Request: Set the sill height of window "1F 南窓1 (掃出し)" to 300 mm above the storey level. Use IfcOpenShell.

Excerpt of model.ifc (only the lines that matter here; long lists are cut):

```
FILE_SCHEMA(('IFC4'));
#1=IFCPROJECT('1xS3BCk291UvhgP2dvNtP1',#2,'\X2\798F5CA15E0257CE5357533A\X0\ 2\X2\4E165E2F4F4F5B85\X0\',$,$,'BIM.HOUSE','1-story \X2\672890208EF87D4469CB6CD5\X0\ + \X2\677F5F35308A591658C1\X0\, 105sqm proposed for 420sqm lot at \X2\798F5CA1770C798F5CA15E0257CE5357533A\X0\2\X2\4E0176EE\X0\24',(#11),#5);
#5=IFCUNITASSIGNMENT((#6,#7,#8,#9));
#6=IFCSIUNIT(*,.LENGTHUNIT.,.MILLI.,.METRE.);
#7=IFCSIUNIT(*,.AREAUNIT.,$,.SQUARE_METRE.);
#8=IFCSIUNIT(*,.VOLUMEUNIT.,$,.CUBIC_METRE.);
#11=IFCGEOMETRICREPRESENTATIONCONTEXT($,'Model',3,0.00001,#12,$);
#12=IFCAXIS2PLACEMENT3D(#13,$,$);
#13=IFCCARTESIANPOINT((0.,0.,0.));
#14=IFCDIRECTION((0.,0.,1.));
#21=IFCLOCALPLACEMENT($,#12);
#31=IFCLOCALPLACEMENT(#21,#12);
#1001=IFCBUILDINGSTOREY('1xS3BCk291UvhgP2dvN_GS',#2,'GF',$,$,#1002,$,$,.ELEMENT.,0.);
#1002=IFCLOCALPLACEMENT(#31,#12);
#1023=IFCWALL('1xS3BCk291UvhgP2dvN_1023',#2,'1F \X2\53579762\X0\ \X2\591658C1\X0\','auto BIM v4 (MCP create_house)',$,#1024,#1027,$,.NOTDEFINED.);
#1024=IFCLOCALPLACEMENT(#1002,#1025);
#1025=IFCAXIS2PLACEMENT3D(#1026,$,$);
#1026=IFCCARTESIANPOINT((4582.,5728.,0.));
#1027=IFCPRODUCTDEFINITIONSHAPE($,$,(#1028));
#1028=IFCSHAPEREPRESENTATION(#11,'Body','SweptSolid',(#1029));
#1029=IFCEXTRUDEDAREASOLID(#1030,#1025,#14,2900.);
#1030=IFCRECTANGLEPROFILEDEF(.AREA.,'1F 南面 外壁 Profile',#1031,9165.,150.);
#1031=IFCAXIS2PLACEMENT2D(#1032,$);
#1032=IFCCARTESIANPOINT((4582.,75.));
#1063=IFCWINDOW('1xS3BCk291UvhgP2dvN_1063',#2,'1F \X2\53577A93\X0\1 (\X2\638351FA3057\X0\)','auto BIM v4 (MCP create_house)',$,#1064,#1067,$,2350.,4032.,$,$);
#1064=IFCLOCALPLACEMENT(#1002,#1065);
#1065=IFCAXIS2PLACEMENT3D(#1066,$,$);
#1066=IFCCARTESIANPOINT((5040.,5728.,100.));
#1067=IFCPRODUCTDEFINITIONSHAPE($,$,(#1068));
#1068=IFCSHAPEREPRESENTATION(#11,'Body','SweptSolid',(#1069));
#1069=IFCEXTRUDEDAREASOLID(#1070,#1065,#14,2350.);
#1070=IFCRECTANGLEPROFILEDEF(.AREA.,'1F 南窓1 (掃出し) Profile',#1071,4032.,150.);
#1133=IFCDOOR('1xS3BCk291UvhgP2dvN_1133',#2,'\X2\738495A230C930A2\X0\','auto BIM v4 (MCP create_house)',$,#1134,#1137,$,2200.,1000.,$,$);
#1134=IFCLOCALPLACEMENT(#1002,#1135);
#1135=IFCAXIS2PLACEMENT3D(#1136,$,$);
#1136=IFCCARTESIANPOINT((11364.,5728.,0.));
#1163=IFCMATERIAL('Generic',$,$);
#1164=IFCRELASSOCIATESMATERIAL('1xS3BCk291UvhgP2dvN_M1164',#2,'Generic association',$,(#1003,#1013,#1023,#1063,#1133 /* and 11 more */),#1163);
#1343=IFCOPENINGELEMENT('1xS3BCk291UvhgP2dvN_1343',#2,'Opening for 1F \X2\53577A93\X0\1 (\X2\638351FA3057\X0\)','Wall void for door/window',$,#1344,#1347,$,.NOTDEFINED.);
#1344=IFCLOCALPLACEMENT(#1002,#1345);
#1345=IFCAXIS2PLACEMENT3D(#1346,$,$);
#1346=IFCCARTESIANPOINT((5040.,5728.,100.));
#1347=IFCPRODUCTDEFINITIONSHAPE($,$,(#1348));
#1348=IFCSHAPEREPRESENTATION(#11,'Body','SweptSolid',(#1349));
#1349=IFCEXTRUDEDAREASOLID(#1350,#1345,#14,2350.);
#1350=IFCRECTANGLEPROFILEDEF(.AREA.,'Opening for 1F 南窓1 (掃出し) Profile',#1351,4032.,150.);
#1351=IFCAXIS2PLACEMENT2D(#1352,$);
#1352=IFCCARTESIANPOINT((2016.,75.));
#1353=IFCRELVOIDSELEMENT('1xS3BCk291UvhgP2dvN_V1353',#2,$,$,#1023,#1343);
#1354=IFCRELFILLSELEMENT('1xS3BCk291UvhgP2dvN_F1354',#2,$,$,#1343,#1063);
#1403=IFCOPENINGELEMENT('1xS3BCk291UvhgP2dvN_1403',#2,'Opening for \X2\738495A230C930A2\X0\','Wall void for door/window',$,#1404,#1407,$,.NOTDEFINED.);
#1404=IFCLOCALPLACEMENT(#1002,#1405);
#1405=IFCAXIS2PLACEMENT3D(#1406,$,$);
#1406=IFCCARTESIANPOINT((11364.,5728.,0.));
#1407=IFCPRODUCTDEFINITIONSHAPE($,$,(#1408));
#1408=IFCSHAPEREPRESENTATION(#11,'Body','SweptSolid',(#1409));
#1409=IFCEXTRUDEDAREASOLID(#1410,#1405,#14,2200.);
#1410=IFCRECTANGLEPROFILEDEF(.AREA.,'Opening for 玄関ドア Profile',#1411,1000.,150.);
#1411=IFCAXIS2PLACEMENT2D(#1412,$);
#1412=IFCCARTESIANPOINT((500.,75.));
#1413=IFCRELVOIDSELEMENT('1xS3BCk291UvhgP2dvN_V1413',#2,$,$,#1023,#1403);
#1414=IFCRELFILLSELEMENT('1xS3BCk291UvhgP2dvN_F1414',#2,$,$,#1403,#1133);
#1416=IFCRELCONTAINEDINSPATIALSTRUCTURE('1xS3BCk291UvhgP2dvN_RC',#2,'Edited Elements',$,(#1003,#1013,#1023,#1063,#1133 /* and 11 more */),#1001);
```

```python
import numpy as np
import ifcopenshell
import ifcopenshell.api.geometry
import ifcopenshell.geom
import ifcopenshell.util.element
import ifcopenshell.util.placement
import ifcopenshell.util.shape
import ifcopenshell.util.unit

model = ifcopenshell.open("model.ifc")
unit_scale = ifcopenshell.util.unit.calculate_unit_scale(model)

window = model.by_guid("1xS3BCk291UvhgP2dvN_1063")
opening = window.FillsVoids[0].RelatingOpeningElement
storey = ifcopenshell.util.element.get_container(window, ifc_class="IfcBuildingStorey")
level = ifcopenshell.util.placement.get_local_placement(storey.ObjectPlacement)[2, 3]

# The opening's origin need not be at the sill, so measure its lowest point.
shape = ifcopenshell.geom.create_shape(ifcopenshell.geom.settings(), opening)
bottom = ifcopenshell.util.shape.get_shape_bottom_elevation(shape, shape.geometry) / unit_scale
dz = level + 300.0 - bottom

shift = np.array([0.0, 0.0, dz])
# The window is not placed relative to its opening, so move both.
for product in (opening, window):
    matrix = ifcopenshell.util.placement.get_local_placement(product.ObjectPlacement)
    matrix[:3, 3] += shift
    ifcopenshell.api.geometry.edit_object_placement(model, product=product, matrix=matrix, is_si=False)

print(f"moved by {dz * unit_scale:+.3f} m")

model.write("model_rev.ifc")
```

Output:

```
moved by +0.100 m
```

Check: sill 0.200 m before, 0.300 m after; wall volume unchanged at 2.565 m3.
